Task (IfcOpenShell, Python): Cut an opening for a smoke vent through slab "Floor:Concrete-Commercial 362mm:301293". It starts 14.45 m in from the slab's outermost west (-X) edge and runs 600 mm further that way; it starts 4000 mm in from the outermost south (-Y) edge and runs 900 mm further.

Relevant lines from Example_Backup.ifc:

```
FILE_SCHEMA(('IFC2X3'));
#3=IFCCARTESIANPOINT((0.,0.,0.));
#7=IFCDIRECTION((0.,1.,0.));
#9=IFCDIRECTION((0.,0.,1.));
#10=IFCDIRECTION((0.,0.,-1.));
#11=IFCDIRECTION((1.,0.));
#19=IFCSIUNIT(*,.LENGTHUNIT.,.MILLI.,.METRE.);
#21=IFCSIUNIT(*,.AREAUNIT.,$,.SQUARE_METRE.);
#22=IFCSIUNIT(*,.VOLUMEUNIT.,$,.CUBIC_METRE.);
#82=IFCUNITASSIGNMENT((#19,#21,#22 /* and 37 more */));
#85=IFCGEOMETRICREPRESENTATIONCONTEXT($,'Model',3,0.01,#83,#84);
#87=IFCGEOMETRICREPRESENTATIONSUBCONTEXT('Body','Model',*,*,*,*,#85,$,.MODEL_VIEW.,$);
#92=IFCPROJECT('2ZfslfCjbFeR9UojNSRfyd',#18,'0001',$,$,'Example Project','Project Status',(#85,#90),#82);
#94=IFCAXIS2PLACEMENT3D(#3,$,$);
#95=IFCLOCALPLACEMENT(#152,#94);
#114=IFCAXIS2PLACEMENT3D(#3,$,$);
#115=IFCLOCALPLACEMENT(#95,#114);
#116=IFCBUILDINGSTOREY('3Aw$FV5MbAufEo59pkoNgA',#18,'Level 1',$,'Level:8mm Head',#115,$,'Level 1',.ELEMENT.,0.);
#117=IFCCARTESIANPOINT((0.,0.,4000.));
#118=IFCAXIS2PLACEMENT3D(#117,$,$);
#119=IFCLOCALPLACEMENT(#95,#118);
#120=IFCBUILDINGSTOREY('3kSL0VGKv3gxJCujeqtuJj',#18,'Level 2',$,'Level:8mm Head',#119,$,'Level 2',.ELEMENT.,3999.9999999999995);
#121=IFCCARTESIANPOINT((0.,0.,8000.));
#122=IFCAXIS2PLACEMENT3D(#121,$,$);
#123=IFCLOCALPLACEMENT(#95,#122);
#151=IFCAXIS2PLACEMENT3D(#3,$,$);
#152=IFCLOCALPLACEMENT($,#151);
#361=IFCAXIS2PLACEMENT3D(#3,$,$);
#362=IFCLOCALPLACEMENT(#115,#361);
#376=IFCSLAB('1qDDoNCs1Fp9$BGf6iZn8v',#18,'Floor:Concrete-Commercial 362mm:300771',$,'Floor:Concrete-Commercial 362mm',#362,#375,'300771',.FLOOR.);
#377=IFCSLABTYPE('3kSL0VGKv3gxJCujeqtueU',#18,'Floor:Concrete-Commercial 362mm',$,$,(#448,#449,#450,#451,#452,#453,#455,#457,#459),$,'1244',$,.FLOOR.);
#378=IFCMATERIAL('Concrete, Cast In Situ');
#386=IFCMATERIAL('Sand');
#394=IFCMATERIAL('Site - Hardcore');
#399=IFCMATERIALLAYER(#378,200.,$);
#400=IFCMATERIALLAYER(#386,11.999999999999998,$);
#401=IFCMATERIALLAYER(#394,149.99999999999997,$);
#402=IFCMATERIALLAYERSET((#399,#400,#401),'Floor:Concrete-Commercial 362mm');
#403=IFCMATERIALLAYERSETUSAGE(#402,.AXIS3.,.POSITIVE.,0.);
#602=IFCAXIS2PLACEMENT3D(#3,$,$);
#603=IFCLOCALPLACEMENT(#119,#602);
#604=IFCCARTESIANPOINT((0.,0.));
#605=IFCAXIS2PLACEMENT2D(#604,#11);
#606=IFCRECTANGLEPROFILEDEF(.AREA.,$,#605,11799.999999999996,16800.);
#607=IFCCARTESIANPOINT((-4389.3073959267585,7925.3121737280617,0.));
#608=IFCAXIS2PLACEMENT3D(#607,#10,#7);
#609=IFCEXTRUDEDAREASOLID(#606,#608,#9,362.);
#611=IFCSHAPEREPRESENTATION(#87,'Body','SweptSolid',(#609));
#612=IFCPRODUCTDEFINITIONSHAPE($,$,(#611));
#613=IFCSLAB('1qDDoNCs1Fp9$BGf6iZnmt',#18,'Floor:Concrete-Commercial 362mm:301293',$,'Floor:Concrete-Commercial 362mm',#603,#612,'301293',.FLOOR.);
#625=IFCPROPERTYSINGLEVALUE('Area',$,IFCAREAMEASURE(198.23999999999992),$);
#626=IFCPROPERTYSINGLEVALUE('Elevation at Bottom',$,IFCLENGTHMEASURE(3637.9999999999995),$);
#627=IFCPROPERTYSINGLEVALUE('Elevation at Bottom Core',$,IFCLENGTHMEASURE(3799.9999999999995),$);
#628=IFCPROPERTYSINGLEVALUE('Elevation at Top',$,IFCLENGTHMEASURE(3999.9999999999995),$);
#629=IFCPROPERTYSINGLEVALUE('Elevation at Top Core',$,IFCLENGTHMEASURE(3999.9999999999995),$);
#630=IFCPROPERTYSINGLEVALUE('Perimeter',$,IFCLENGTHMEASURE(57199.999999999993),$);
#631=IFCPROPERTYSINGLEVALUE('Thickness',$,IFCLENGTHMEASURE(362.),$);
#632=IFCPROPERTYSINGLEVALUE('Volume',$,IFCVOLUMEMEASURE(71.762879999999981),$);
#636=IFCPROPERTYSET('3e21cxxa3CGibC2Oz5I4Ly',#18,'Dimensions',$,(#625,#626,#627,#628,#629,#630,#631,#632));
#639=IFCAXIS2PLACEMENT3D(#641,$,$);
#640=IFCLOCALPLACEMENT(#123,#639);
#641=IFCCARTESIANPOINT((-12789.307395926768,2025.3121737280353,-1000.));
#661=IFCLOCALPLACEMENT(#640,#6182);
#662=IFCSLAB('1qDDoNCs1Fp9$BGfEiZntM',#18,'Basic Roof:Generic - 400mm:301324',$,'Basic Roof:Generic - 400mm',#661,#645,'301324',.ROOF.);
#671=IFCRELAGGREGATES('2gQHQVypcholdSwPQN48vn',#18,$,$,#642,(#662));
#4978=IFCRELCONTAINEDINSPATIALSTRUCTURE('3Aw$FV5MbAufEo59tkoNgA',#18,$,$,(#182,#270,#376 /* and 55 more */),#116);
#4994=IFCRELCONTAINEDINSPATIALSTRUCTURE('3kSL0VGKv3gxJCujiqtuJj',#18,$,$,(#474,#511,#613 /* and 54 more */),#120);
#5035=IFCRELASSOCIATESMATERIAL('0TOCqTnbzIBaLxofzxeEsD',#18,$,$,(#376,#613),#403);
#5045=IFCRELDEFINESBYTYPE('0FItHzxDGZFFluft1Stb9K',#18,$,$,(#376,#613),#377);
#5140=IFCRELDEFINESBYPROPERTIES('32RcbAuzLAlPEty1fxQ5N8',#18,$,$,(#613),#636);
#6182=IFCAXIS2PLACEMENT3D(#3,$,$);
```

```python
import numpy as np
import ifcopenshell
import ifcopenshell.api.feature
import ifcopenshell.api.geometry
import ifcopenshell.api.pset
import ifcopenshell.api.root
import ifcopenshell.geom
import ifcopenshell.util.element
import ifcopenshell.util.placement
import ifcopenshell.util.representation
import ifcopenshell.util.shape
import ifcopenshell.util.unit

model = ifcopenshell.open("Example_Backup.ifc")
unit_scale = ifcopenshell.util.unit.calculate_unit_scale(model)
area_scale = ifcopenshell.util.unit.calculate_unit_scale(model, "AREAUNIT")
volume_scale = ifcopenshell.util.unit.calculate_unit_scale(model, "VOLUMEUNIT")
settings = ifcopenshell.geom.settings()


def volume(element):
    """Net volume in cubic metres, openings subtracted."""
    shape = ifcopenshell.geom.create_shape(settings, element)
    return ifcopenshell.util.shape.get_volume(shape.geometry)


slab = model.by_guid("1qDDoNCs1Fp9$BGf6iZnmt")
before = volume(slab)

# Extent in the slab's own axes, in metres. The edges named are its -X and -Y sides.
slab_shape = ifcopenshell.geom.create_shape(settings, slab)
vertices = ifcopenshell.util.shape.get_vertices(slab_shape.geometry)
x_min, y_min, bottom = vertices.min(axis=0)
top = vertices[:, 2].max()

opening = ifcopenshell.api.root.create_entity(model, ifc_class="IfcOpeningElement", name="Smoke vent opening")
context = ifcopenshell.util.representation.get_context(model, "Model", "Body", "MODEL_VIEW")
width, depth = 0.6, 0.9
outline = [(0.0, 0.0), (width, 0.0), (width, depth), (0.0, depth), (0.0, 0.0)]
# Overshoot both faces by 50 mm so the cut is clean.
shape = ifcopenshell.api.geometry.add_slab_representation(
    model, context=context, depth=top - bottom + 0.1, polyline=outline
)
ifcopenshell.api.geometry.assign_representation(model, product=opening, representation=shape)

matrix = ifcopenshell.util.placement.get_local_placement(slab.ObjectPlacement)
matrix[:, 3] = matrix @ np.append(np.array([x_min + 14.45, y_min + 4, bottom - 0.05]) / unit_scale, 1.0)
ifcopenshell.api.geometry.edit_object_placement(model, product=opening, matrix=matrix, is_si=False)
ifcopenshell.api.feature.add_feature(model, feature=opening, element=slab)

after = volume(slab)

# Update the slab's stored quantities.
pset = model.by_id(ifcopenshell.util.element.get_pset(slab, "Dimensions", should_inherit=False)["id"])
ifcopenshell.api.pset.edit_pset(model, pset=pset, properties={
    "Area": model.create_entity("IfcAreaMeasure", after / (top - bottom) / area_scale),
    "Volume": model.create_entity("IfcVolumeMeasure", after / volume_scale),
})

print(f"slab volume {before:.3f} -> {after:.3f} m3")

model.write("Example_Backup_edited.ifc")
```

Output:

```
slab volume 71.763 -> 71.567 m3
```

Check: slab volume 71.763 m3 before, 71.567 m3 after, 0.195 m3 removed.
